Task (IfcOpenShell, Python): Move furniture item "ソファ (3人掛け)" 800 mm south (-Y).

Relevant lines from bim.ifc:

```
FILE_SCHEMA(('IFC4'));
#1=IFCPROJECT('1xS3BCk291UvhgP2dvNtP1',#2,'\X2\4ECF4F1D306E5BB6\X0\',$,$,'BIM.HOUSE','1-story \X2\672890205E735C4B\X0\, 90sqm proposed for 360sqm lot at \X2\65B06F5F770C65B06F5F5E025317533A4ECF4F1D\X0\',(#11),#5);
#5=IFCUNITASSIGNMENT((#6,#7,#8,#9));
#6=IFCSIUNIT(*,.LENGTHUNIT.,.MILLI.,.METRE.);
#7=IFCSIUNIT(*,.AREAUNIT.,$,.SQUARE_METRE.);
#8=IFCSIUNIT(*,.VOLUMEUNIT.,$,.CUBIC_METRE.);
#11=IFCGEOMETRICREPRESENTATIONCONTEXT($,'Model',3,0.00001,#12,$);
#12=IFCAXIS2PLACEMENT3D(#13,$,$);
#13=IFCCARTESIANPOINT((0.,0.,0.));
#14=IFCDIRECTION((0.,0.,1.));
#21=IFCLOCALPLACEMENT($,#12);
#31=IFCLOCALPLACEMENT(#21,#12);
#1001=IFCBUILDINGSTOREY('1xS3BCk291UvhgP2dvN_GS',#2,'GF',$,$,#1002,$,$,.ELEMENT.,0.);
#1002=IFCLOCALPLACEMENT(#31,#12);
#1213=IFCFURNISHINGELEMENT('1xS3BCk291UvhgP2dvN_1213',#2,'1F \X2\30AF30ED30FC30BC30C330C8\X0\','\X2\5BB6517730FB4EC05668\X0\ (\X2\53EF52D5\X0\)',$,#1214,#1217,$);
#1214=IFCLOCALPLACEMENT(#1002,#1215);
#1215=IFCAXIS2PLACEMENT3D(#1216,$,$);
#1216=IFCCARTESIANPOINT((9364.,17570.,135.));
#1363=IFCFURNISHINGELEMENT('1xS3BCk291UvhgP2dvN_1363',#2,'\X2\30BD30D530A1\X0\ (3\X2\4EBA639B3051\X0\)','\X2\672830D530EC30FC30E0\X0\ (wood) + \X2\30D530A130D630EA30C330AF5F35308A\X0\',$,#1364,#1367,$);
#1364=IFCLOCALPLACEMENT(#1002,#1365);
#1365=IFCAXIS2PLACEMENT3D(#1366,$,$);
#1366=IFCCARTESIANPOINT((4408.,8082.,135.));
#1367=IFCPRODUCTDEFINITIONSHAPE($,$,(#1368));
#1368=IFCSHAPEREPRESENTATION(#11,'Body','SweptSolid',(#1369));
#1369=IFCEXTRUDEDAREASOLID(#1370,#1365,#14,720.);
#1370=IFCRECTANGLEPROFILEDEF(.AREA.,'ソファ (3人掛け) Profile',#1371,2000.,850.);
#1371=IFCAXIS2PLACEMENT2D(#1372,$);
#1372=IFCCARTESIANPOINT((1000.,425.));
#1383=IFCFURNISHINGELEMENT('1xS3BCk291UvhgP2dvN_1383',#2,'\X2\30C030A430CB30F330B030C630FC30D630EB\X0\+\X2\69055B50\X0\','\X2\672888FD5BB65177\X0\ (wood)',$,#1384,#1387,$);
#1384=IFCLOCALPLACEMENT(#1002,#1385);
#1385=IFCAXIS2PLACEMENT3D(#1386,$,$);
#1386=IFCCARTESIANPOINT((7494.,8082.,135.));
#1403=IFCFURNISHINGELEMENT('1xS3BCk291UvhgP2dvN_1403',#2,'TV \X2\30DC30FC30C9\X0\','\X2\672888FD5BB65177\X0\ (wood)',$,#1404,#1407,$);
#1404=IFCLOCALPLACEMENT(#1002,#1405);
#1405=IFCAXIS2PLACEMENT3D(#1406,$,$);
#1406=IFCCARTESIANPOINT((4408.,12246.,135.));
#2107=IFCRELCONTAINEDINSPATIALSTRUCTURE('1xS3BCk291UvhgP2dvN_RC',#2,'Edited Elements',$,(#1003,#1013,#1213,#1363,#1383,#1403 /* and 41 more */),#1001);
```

```python
import ifcopenshell
import ifcopenshell.api.geometry
import ifcopenshell.util.placement
import ifcopenshell.util.unit

model = ifcopenshell.open("bim.ifc")
unit_scale = ifcopenshell.util.unit.calculate_unit_scale(model)

item = model.by_guid("1xS3BCk291UvhgP2dvN_1363")
matrix = ifcopenshell.util.placement.get_local_placement(item.ObjectPlacement)
matrix[1, 3] -= 0.8 / unit_scale
ifcopenshell.api.geometry.edit_object_placement(model, product=item, matrix=matrix, is_si=False)

print(ifcopenshell.util.placement.get_local_placement(item.ObjectPlacement).round(3) + 0.0)

model.write("bim_updated.ifc")
```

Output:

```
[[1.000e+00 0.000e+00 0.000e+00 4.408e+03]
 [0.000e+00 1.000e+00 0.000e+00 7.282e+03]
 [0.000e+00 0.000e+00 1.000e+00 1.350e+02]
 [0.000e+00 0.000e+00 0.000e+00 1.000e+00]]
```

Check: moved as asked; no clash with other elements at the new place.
